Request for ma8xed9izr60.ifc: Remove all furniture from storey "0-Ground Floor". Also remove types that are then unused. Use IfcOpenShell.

First a look at what the model holds.

```python
import ifcopenshell
import ifcopenshell.util.element

model = ifcopenshell.open("ma8xed9izr60.ifc")
print(model.schema)
storey = next(s for s in model.by_type("IfcBuildingStorey") if s.Name == "0-Ground Floor")
furniture = [e for e in ifcopenshell.util.element.get_decomposition(storey) if e.is_a("IfcFurnishingElement")]
seen = {}
for e in furniture:
    element_type = ifcopenshell.util.element.get_type(e)
    name = element_type.Name if element_type not in (None, e) else None
    seen[name] = seen.get(name, 0) + 1
for name, count in sorted(seen.items(), key=str):
    print(count, "x", name)
```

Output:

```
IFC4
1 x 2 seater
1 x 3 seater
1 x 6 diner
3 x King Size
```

```python
import ifcopenshell
import ifcopenshell.api.root
import ifcopenshell.util.element

model = ifcopenshell.open("ma8xed9izr60.ifc")

storey = next(s for s in model.by_type("IfcBuildingStorey") if s.Name == "0-Ground Floor")
furniture = [e for e in ifcopenshell.util.element.get_decomposition(storey) if e.is_a("IfcFurnishingElement")]
types = {ifcopenshell.util.element.get_type(e) for e in furniture} - {None, *furniture}

for e in furniture:
    ifcopenshell.api.root.remove_product(model, product=e)
print(len(furniture), "removed")

unused = [t for t in types if not ifcopenshell.util.element.get_types(t)]
for t in unused:
    ifcopenshell.api.root.remove_product(model, product=t)
print(len(unused), "unused types removed")

model.write("ma8xed9izr60_updated.ifc")
```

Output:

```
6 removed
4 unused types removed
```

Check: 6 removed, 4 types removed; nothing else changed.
